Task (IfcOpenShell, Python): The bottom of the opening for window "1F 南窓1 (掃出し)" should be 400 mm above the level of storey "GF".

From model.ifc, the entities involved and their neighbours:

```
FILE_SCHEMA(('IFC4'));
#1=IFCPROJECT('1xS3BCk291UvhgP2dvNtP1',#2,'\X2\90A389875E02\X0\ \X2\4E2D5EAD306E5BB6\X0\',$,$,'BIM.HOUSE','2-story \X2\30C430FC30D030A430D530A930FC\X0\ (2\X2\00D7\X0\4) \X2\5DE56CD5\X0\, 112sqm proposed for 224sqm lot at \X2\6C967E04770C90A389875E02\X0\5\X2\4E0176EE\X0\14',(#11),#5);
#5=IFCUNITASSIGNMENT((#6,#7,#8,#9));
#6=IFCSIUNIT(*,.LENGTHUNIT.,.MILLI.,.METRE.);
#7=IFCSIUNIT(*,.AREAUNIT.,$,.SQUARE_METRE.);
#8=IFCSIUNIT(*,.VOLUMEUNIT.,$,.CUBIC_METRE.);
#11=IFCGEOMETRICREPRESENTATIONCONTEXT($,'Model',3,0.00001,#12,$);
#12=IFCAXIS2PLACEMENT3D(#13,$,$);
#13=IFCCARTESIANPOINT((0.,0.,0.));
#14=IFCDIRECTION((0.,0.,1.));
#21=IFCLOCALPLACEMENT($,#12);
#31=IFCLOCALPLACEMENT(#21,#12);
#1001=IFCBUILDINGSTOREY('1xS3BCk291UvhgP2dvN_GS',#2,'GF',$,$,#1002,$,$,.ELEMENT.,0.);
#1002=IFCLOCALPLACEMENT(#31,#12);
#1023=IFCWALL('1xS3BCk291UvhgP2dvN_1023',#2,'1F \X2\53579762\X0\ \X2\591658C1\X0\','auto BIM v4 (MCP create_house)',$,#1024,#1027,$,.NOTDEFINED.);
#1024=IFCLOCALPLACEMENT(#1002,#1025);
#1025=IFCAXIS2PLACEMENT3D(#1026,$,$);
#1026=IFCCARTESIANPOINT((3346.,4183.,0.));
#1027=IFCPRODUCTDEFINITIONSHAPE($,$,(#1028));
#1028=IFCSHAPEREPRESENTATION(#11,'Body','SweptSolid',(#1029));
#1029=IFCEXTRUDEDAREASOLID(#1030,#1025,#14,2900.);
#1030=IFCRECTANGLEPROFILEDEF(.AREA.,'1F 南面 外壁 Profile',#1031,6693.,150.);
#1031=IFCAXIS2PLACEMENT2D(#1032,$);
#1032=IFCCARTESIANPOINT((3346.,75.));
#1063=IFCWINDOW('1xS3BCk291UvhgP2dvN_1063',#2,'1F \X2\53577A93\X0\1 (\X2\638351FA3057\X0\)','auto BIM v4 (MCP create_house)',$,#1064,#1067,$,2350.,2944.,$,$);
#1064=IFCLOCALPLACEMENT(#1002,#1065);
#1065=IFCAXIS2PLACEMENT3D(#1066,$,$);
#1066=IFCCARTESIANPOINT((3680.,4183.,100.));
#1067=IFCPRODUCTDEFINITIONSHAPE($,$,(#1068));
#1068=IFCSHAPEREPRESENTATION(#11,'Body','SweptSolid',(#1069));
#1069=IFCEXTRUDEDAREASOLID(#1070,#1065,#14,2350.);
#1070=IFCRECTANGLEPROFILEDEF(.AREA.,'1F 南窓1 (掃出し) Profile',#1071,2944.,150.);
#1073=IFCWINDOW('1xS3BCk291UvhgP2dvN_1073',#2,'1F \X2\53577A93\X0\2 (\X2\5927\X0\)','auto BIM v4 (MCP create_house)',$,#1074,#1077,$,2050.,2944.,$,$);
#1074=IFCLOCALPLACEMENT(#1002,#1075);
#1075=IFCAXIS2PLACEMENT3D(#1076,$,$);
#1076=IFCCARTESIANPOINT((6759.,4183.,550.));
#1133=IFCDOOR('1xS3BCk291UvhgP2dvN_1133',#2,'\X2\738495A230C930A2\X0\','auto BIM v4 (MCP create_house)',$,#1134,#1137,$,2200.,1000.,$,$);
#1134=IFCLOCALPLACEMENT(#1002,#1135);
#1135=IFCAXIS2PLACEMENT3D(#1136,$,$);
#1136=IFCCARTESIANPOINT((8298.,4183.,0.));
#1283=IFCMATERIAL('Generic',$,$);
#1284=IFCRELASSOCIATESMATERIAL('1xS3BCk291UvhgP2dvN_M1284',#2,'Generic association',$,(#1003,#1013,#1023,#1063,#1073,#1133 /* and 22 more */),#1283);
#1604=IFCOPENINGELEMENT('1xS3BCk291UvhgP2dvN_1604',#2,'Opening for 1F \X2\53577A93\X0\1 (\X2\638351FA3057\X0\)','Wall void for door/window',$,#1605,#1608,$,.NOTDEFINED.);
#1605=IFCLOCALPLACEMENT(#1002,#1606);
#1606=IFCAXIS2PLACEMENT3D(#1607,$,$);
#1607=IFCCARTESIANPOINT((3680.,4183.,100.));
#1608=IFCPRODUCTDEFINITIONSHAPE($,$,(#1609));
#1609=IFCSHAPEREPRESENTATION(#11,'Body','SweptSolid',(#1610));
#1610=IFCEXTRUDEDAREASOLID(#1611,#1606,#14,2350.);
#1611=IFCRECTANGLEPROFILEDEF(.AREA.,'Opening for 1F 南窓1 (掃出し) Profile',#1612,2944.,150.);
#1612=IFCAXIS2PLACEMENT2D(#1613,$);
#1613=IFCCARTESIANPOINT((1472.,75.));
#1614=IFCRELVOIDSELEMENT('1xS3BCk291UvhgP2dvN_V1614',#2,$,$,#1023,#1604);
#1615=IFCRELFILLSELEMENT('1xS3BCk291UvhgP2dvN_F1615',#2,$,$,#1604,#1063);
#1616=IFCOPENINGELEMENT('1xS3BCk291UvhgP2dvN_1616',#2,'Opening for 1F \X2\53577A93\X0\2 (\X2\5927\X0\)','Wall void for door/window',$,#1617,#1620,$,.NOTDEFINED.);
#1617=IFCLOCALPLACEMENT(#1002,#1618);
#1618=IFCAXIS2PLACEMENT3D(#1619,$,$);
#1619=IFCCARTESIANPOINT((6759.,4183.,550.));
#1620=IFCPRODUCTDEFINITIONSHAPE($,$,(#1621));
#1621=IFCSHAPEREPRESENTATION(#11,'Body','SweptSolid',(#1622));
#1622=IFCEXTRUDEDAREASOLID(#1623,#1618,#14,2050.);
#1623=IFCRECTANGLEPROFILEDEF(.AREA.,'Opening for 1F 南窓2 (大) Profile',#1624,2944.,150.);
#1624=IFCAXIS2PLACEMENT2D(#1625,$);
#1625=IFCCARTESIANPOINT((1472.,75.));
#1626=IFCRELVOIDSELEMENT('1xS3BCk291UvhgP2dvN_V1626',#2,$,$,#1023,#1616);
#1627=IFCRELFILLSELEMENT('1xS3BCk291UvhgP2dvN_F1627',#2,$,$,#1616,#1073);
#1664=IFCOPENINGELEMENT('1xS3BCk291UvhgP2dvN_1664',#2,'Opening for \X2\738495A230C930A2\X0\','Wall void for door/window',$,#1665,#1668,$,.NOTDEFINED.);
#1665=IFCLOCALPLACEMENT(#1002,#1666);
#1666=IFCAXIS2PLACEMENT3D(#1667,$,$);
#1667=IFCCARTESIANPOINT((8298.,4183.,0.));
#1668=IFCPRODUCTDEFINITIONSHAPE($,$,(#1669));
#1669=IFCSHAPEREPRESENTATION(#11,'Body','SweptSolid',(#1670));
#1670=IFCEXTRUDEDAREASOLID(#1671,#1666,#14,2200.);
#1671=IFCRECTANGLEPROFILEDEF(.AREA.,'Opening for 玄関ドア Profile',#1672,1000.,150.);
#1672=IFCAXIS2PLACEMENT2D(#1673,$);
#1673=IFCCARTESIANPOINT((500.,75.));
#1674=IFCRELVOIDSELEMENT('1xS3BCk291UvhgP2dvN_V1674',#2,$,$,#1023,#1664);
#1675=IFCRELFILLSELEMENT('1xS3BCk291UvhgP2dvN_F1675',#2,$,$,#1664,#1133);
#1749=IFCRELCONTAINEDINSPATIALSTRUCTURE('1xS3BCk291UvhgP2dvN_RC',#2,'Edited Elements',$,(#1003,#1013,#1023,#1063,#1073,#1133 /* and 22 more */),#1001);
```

```python
import numpy as np
import ifcopenshell
import ifcopenshell.api.geometry
import ifcopenshell.geom
import ifcopenshell.util.element
import ifcopenshell.util.placement
import ifcopenshell.util.shape
import ifcopenshell.util.unit

model = ifcopenshell.open("model.ifc")
unit_scale = ifcopenshell.util.unit.calculate_unit_scale(model)

window = model.by_guid("1xS3BCk291UvhgP2dvN_1063")
opening = window.FillsVoids[0].RelatingOpeningElement
storey = ifcopenshell.util.element.get_container(window, ifc_class="IfcBuildingStorey")
level = ifcopenshell.util.placement.get_local_placement(storey.ObjectPlacement)[2, 3]

# The opening's origin need not be at the sill, so measure its lowest point.
shape = ifcopenshell.geom.create_shape(ifcopenshell.geom.settings(), opening)
bottom = ifcopenshell.util.shape.get_shape_bottom_elevation(shape, shape.geometry) / unit_scale
dz = level + 0.4 / unit_scale - bottom

shift = np.array([0.0, 0.0, dz])
# The window is not placed relative to its opening, so move both.
for product in (opening, window):
    matrix = ifcopenshell.util.placement.get_local_placement(product.ObjectPlacement)
    matrix[:3, 3] += shift
    ifcopenshell.api.geometry.edit_object_placement(model, product=product, matrix=matrix, is_si=False)

print(f"moved by {dz * unit_scale:+.3f} m")

model.write("model-out.ifc")
```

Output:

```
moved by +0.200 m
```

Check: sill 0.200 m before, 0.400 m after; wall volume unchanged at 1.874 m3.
